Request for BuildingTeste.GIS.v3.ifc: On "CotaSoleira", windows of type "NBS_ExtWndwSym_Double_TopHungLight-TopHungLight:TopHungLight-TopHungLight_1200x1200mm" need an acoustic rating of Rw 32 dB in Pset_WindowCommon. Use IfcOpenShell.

First a look at what the model holds.

```python
import ifcopenshell
import ifcopenshell.util.element

model = ifcopenshell.open("BuildingTeste.GIS.v3.ifc")
print(model.schema)
storey = next(s for s in model.by_type("IfcBuildingStorey") if s.Name == "CotaSoleira")
windows = [e for e in ifcopenshell.util.element.get_decomposition(storey) if e.is_a("IfcWindow")]
seen = {}
for e in windows:
    element_type = ifcopenshell.util.element.get_type(e)
    key = (element_type.Name if element_type != e and element_type else None, ifcopenshell.util.element.get_pset(e, "Pset_WindowCommon", "AcousticRating"))
    seen[key] = seen.get(key, 0) + 1
for (name, value), count in sorted(seen.items(), key=str):
    print(count, "x", name, "|", value)
```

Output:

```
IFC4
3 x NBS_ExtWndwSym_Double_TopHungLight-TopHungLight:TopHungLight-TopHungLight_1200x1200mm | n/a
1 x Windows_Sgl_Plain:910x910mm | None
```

```python
import ifcopenshell
import ifcopenshell.api.pset
import ifcopenshell.util.element

model = ifcopenshell.open("BuildingTeste.GIS.v3.ifc")

storey = next(s for s in model.by_type("IfcBuildingStorey") if s.Name == "CotaSoleira")
windows = [e for e in ifcopenshell.util.element.get_decomposition(storey) if e.is_a("IfcWindow")]

count = 0
for e in windows:
    element_type = ifcopenshell.util.element.get_type(e)
    if element_type in (None, e) or element_type.Name != "NBS_ExtWndwSym_Double_TopHungLight-TopHungLight:TopHungLight-TopHungLight_1200x1200mm":
        continue
    # add_pset returns the element's existing set when there is one.
    pset = ifcopenshell.api.pset.add_pset(model, product=e, name="Pset_WindowCommon")
    ifcopenshell.api.pset.edit_pset(model, pset=pset, properties={"AcousticRating": "Rw 32 dB"})
    count += 1

print(count, "windows updated")

model.write("BuildingTeste.GIS.v3-out.ifc")
```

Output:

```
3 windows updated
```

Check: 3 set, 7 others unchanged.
